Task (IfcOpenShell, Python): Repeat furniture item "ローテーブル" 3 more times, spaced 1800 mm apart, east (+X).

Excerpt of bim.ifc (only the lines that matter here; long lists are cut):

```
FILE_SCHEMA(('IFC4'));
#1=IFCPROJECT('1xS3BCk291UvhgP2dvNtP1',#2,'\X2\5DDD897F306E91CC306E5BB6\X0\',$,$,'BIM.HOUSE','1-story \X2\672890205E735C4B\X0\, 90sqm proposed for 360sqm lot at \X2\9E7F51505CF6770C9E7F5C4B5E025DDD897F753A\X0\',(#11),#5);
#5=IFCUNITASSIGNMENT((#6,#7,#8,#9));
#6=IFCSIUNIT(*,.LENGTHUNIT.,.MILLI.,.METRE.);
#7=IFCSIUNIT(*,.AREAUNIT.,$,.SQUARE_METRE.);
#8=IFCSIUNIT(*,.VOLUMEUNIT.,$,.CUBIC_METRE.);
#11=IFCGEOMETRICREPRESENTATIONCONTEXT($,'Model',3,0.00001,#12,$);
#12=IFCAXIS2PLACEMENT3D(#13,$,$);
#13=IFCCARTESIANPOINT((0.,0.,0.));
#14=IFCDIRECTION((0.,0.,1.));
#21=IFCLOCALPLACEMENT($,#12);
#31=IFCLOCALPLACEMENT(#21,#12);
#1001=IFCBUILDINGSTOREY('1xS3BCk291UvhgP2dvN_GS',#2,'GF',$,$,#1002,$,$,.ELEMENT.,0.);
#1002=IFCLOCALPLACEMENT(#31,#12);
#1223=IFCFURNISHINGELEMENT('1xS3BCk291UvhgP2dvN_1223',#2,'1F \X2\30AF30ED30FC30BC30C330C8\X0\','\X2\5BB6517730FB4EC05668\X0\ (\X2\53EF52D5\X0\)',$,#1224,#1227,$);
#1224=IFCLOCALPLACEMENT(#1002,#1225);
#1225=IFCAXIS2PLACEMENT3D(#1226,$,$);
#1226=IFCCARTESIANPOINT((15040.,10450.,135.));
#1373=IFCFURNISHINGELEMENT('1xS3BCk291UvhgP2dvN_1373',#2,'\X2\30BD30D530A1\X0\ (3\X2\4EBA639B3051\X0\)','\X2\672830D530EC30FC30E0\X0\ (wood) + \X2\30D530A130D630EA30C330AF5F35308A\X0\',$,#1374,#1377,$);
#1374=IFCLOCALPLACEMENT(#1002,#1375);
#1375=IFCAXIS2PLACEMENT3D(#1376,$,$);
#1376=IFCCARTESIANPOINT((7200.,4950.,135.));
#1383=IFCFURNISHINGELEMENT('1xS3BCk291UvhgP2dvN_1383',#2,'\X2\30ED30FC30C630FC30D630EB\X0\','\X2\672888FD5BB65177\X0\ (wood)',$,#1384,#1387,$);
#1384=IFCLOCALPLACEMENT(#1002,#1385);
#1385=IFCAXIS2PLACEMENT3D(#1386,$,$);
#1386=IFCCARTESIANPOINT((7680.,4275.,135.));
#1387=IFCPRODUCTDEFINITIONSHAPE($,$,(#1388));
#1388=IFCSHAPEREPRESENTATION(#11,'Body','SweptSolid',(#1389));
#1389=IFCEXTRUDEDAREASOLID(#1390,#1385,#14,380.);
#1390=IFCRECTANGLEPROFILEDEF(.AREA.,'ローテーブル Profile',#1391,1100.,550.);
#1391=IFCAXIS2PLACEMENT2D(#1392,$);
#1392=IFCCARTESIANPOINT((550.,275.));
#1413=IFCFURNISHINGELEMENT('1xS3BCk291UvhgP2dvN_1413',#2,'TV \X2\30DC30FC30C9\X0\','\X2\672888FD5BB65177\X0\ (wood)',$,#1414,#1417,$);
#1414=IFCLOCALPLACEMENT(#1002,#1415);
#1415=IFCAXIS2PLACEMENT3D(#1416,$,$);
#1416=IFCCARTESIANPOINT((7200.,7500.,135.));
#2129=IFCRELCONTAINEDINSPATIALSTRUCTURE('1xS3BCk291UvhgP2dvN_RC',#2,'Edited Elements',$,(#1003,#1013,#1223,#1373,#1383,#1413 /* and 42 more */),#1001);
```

```python
import numpy as np
import ifcopenshell
import ifcopenshell.api.geometry
import ifcopenshell.api.root
import ifcopenshell.util.element
import ifcopenshell.util.placement

model = ifcopenshell.open("bim.ifc")


def reuse_history(source, copy):
    """copy_class also copies each property set's owner history, people and application; keep the originals."""
    for rel in copy.IsDefinedBy:
        if rel.is_a("IfcRelDefinesByProperties") and (history := rel.RelatingPropertyDefinition.OwnerHistory):
            rel.RelatingPropertyDefinition.OwnerHistory = source.OwnerHistory
            ifcopenshell.util.element.remove_deep2(model, history)


source = model.by_guid("1xS3BCk291UvhgP2dvN_1383")
base = ifcopenshell.util.placement.get_local_placement(source.ObjectPlacement)
step = np.array([1.0, 0.0, 0.0]) * 1800.0

for i in range(1, 4):
    copy = ifcopenshell.api.root.copy_class(model, product=source)
    copy.Representation = ifcopenshell.util.element.copy_deep(
        model, source.Representation, exclude=["IfcGeometricRepresentationContext", "IfcRepresentationMap"]
    )
    reuse_history(source, copy)
    matrix = base.copy()
    matrix[:3, 3] += i * step
    print("added at", matrix[:3, 3].round(3) + 0.0)
    ifcopenshell.api.geometry.edit_object_placement(model, product=copy, matrix=matrix, is_si=False)

model.write("bim_rev.ifc")
```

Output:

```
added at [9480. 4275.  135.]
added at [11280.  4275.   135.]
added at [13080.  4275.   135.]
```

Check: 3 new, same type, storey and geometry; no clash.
